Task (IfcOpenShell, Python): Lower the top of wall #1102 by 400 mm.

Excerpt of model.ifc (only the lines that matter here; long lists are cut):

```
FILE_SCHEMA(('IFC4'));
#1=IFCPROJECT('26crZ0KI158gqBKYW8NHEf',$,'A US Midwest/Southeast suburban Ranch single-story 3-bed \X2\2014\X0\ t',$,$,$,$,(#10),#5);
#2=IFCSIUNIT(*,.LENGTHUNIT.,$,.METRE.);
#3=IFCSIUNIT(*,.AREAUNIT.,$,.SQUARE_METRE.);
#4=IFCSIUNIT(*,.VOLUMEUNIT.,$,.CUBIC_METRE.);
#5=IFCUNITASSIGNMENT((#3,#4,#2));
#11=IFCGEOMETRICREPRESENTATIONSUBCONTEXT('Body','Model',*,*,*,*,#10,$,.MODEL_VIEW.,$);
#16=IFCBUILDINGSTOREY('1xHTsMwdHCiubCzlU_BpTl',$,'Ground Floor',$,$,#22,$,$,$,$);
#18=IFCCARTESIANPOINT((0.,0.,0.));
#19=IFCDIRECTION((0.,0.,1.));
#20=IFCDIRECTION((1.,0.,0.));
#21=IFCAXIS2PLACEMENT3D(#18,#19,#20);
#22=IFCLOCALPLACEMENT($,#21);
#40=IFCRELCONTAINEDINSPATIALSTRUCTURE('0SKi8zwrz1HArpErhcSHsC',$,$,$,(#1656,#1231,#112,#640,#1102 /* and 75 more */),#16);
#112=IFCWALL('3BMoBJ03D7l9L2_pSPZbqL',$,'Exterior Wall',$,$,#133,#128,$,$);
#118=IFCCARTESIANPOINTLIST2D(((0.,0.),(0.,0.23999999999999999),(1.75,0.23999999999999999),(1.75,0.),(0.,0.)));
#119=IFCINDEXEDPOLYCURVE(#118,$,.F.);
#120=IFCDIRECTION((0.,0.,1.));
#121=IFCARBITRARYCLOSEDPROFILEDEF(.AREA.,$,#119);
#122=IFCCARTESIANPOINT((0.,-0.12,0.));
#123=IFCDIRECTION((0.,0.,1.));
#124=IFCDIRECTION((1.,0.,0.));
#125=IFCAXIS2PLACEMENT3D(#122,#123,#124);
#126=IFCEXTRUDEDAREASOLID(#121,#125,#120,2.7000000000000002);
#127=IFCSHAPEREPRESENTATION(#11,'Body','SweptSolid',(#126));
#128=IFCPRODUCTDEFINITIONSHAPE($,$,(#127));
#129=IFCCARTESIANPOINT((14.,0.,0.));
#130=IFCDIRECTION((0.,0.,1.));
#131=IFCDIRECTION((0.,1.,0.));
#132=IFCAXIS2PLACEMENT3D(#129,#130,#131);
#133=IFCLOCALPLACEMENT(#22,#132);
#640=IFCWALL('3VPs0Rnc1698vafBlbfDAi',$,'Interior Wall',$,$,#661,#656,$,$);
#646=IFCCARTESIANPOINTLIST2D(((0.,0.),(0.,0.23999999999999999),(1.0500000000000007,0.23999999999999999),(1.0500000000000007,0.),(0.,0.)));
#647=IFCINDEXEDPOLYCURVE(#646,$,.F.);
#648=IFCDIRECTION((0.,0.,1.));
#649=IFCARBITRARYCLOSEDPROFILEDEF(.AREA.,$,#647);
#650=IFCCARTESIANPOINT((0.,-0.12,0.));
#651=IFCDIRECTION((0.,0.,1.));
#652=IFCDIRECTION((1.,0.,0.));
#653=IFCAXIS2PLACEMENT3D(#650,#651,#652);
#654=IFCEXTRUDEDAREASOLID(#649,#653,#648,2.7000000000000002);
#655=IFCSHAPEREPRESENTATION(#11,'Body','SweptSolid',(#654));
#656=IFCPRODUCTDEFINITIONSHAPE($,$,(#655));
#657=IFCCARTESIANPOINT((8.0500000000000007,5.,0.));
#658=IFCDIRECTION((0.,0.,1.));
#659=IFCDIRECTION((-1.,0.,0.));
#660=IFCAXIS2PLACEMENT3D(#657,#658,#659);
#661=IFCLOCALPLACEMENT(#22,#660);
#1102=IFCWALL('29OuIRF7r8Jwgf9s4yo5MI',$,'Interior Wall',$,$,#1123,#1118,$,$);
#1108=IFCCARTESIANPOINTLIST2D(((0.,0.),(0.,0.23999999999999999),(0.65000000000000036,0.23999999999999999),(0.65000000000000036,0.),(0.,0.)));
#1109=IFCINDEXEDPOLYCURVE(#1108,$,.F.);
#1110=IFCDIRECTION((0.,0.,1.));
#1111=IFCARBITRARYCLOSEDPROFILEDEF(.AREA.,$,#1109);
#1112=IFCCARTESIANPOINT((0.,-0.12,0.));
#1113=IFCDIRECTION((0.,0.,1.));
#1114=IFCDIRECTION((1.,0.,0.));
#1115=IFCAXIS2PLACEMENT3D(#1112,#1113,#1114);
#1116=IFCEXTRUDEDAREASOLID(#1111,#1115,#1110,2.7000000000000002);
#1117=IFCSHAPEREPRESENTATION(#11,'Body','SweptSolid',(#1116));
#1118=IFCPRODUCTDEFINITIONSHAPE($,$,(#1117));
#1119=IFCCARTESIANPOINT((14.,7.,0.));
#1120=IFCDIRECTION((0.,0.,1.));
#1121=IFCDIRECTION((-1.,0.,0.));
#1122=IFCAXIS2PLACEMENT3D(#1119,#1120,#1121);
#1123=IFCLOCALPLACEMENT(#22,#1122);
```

```python
import ifcopenshell
import ifcopenshell.geom
import ifcopenshell.util.representation
import ifcopenshell.util.shape
import ifcopenshell.util.unit

model = ifcopenshell.open("model.ifc")
unit_scale = ifcopenshell.util.unit.calculate_unit_scale(model)
settings = ifcopenshell.geom.settings()


def volume(element):
    """Net volume in cubic metres, openings subtracted."""
    shape = ifcopenshell.geom.create_shape(settings, element)
    return ifcopenshell.util.shape.get_volume(shape.geometry)


wall = model.by_guid("29OuIRF7r8Jwgf9s4yo5MI")
before = volume(wall)

body = ifcopenshell.util.representation.get_representation(wall, "Model", "Body")
solid = body.Items[0]
old_height = solid.Depth
solid.Depth -= 0.4 / unit_scale
after = volume(wall)

print(f"height {old_height:g} -> {solid.Depth:g}, volume {before:.3f} -> {after:.3f} m3")

model.write("model-out.ifc")
```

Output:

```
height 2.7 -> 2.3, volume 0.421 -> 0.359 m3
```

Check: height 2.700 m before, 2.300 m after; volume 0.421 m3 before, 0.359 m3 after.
